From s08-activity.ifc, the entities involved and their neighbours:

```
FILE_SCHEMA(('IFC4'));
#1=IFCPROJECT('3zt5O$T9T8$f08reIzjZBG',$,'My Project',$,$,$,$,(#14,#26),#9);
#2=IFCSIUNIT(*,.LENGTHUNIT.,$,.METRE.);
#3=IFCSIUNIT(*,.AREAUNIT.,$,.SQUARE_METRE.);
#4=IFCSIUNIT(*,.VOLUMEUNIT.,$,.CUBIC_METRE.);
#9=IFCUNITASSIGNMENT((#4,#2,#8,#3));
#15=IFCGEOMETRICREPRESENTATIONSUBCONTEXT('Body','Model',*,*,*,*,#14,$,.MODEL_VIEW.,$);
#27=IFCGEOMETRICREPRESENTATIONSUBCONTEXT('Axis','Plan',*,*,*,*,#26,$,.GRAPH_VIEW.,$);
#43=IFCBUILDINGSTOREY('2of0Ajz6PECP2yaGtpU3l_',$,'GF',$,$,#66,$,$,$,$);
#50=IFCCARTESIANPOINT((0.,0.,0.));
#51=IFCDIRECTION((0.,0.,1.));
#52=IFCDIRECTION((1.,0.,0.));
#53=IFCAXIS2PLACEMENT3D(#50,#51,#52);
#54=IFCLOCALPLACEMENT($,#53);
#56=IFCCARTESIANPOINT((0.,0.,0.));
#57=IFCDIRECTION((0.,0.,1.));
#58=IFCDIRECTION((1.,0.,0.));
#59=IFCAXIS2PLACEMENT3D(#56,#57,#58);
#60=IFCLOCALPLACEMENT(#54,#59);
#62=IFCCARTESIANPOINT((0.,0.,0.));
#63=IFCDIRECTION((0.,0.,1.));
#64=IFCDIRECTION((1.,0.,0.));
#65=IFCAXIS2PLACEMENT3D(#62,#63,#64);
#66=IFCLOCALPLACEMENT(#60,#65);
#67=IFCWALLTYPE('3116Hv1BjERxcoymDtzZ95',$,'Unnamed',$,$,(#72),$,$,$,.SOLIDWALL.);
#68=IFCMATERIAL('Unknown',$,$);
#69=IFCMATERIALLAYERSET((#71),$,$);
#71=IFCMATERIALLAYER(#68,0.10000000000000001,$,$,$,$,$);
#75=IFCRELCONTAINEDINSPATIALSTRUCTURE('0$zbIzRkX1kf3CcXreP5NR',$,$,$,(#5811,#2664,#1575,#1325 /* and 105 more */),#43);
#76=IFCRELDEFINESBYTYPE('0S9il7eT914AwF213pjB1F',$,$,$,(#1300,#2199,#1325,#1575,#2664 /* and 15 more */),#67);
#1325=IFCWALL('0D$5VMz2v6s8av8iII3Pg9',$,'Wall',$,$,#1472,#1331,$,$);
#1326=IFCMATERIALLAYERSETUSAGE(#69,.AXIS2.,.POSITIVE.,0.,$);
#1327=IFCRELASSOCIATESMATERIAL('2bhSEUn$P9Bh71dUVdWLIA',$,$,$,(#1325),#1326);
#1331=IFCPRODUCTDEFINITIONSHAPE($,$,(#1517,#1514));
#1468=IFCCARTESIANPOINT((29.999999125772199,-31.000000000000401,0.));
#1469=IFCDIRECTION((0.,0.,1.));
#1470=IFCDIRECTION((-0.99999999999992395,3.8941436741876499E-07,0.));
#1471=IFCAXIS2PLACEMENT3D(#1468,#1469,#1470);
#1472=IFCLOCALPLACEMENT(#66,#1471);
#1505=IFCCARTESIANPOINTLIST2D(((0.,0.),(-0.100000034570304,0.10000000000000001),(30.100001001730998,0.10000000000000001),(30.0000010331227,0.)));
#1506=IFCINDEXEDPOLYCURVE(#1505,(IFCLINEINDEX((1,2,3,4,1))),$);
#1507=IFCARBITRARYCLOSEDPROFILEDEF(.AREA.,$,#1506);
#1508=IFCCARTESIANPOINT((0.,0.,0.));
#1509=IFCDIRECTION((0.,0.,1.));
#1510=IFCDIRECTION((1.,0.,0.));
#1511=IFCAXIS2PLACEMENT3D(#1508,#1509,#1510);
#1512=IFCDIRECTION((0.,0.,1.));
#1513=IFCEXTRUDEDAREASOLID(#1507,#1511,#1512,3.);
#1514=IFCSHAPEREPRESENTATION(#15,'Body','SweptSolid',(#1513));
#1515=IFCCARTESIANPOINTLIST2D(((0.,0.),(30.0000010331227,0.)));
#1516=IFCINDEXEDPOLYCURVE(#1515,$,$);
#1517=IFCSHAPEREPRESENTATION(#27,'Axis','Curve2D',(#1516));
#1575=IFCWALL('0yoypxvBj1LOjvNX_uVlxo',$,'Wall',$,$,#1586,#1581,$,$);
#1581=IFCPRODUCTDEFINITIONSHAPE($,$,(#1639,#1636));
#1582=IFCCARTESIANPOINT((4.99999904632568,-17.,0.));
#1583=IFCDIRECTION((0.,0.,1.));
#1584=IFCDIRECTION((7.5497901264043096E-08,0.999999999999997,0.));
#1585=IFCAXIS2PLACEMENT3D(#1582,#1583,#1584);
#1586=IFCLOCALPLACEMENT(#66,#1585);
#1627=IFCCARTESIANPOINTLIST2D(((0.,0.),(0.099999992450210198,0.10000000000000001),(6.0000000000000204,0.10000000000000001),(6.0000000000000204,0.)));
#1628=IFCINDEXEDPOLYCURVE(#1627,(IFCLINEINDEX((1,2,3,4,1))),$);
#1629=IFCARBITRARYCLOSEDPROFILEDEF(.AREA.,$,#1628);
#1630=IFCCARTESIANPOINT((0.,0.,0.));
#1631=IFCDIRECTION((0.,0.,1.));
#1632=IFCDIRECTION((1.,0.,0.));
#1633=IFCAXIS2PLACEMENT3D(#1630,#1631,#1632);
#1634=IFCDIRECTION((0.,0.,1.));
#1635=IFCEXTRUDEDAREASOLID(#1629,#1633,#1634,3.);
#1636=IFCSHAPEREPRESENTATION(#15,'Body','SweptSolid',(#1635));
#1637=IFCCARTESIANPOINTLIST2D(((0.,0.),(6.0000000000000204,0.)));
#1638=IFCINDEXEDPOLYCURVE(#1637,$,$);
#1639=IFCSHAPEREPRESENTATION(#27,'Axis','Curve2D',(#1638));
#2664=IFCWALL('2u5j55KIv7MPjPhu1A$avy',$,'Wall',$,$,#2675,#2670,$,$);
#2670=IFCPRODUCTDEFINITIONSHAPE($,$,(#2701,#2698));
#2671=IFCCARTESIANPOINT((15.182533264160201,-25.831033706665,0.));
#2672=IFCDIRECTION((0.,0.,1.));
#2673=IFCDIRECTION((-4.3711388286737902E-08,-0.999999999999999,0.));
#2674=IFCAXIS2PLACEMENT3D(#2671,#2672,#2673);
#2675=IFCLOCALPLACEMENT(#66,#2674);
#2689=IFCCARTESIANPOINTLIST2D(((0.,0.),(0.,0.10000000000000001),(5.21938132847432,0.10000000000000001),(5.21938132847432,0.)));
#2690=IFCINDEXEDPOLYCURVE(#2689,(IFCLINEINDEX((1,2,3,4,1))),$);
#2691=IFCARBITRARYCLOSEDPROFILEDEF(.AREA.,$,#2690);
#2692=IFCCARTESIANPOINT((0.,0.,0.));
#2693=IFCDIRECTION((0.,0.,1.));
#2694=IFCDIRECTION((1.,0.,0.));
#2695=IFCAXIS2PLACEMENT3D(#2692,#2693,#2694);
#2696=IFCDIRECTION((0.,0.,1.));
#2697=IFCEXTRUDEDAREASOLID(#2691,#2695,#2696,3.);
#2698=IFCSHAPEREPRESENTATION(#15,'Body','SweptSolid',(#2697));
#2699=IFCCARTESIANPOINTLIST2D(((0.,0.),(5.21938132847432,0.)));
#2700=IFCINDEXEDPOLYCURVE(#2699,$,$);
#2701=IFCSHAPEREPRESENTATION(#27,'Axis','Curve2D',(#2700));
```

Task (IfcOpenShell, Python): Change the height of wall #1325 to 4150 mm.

```python
import ifcopenshell
import ifcopenshell.geom
import ifcopenshell.util.representation
import ifcopenshell.util.shape

model = ifcopenshell.open("s08-activity.ifc")
settings = ifcopenshell.geom.settings()


def volume(element):
    """Net volume in cubic metres, openings subtracted."""
    shape = ifcopenshell.geom.create_shape(settings, element)
    return ifcopenshell.util.shape.get_volume(shape.geometry)


wall = model.by_guid("0D$5VMz2v6s8av8iII3Pg9")
before = volume(wall)

body = ifcopenshell.util.representation.get_representation(wall, "Model", "Body")
solid = body.Items[0]
old_height = solid.Depth
solid.Depth = 4.15
after = volume(wall)

print(f"height {old_height:g} -> {solid.Depth:g}, volume {before:.3f} -> {after:.3f} m3")

model.write("s08-activity-out.ifc")
```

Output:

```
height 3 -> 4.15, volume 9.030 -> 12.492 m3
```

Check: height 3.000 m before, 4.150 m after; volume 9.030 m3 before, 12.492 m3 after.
